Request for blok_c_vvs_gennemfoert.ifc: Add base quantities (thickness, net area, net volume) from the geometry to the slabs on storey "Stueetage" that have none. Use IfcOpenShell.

First a look at what the model holds.

```python
import ifcopenshell
import ifcopenshell.util.element
import ifcopenshell.util.unit

model = ifcopenshell.open("blok_c_vvs_gennemfoert.ifc")
print(model.schema)
for unit_type in ("LENGTHUNIT", "AREAUNIT", "VOLUMEUNIT"):
    print(unit_type, ifcopenshell.util.unit.calculate_unit_scale(model, unit_type))
storey = next(s for s in model.by_type("IfcBuildingStorey") if s.Name == "Stueetage")
slabs = [e for e in ifcopenshell.util.element.get_decomposition(storey) if e.is_a("IfcSlab")]
for e in sorted(slabs, key=lambda e: e.id()):
    print(e.id(), e.is_a(), e.Name, list(ifcopenshell.util.element.get_psets(e, qtos_only=True)), sep=" | ")
```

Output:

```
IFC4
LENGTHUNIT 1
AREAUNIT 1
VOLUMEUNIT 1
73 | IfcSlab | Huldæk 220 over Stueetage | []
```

```python
import ifcopenshell
import ifcopenshell.api.pset
import ifcopenshell.geom
import ifcopenshell.util.element
import ifcopenshell.util.shape
import ifcopenshell.util.unit

model = ifcopenshell.open("blok_c_vvs_gennemfoert.ifc")
unit_scale = ifcopenshell.util.unit.calculate_unit_scale(model)
area_scale = ifcopenshell.util.unit.calculate_unit_scale(model, "AREAUNIT")
volume_scale = ifcopenshell.util.unit.calculate_unit_scale(model, "VOLUMEUNIT")
settings = ifcopenshell.geom.settings()

storey = next(s for s in model.by_type("IfcBuildingStorey") if s.Name == "Stueetage")
slabs = [e for e in ifcopenshell.util.element.get_decomposition(storey) if e.is_a("IfcSlab")]

for e in sorted(slabs, key=lambda e: e.id()):
    if ifcopenshell.util.element.get_psets(e, qtos_only=True, should_inherit=False):
        continue
    # Geometry comes back in metres, in the element's own axes.
    shape = ifcopenshell.geom.create_shape(settings, e)
    values = {
        "Width": ifcopenshell.util.shape.get_z(shape.geometry) / unit_scale,
        "NetArea": ifcopenshell.util.shape.get_footprint_area(shape.geometry) / area_scale,
        "NetVolume": ifcopenshell.util.shape.get_volume(shape.geometry) / volume_scale,
    }
    qto = ifcopenshell.api.pset.add_qto(model, product=e, name="Qto_SlabBaseQuantities")
    ifcopenshell.api.pset.edit_qto(model, qto=qto, properties=values)
    print(e.id(), {k: round(v, 3) for k, v in values.items()})

model.write("blok_c_vvs_gennemfoert_v2.ifc")
```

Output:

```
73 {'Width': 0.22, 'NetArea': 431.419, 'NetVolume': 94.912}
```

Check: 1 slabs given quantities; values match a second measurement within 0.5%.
